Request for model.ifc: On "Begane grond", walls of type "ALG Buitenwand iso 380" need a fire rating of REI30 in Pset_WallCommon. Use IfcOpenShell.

First a look at what the model holds.

```python
import ifcopenshell
import ifcopenshell.util.element

model = ifcopenshell.open("model.ifc")
print(model.schema)
storey = next(s for s in model.by_type("IfcBuildingStorey") if s.Name == "Begane grond")
walls = [e for e in ifcopenshell.util.element.get_decomposition(storey) if e.is_a("IfcWall")]
seen = {}
for e in walls:
    element_type = ifcopenshell.util.element.get_type(e)
    key = (element_type.Name if element_type != e and element_type else None, ifcopenshell.util.element.get_pset(e, "Pset_WallCommon", "FireRating"))
    seen[key] = seen.get(key, 0) + 1
for (name, value), count in sorted(seen.items(), key=str):
    print(count, "x", name, "|", value)
```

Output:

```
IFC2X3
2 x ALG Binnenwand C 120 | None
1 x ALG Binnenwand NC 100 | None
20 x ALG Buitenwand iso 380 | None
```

```python
import ifcopenshell
import ifcopenshell.api.pset
import ifcopenshell.util.element

model = ifcopenshell.open("model.ifc")

storey = next(s for s in model.by_type("IfcBuildingStorey") if s.Name == "Begane grond")
walls = [e for e in ifcopenshell.util.element.get_decomposition(storey) if e.is_a("IfcWall")]

count = 0
for e in walls:
    element_type = ifcopenshell.util.element.get_type(e)
    if element_type in (None, e) or element_type.Name != "ALG Buitenwand iso 380":
        continue
    # add_pset returns the element's existing set when there is one.
    pset = ifcopenshell.api.pset.add_pset(model, product=e, name="Pset_WallCommon")
    ifcopenshell.api.pset.edit_pset(model, pset=pset, properties={"FireRating": "REI30"})
    count += 1

print(count, "walls updated")

model.write("model-out.ifc")
```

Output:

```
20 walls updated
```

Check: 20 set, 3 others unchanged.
